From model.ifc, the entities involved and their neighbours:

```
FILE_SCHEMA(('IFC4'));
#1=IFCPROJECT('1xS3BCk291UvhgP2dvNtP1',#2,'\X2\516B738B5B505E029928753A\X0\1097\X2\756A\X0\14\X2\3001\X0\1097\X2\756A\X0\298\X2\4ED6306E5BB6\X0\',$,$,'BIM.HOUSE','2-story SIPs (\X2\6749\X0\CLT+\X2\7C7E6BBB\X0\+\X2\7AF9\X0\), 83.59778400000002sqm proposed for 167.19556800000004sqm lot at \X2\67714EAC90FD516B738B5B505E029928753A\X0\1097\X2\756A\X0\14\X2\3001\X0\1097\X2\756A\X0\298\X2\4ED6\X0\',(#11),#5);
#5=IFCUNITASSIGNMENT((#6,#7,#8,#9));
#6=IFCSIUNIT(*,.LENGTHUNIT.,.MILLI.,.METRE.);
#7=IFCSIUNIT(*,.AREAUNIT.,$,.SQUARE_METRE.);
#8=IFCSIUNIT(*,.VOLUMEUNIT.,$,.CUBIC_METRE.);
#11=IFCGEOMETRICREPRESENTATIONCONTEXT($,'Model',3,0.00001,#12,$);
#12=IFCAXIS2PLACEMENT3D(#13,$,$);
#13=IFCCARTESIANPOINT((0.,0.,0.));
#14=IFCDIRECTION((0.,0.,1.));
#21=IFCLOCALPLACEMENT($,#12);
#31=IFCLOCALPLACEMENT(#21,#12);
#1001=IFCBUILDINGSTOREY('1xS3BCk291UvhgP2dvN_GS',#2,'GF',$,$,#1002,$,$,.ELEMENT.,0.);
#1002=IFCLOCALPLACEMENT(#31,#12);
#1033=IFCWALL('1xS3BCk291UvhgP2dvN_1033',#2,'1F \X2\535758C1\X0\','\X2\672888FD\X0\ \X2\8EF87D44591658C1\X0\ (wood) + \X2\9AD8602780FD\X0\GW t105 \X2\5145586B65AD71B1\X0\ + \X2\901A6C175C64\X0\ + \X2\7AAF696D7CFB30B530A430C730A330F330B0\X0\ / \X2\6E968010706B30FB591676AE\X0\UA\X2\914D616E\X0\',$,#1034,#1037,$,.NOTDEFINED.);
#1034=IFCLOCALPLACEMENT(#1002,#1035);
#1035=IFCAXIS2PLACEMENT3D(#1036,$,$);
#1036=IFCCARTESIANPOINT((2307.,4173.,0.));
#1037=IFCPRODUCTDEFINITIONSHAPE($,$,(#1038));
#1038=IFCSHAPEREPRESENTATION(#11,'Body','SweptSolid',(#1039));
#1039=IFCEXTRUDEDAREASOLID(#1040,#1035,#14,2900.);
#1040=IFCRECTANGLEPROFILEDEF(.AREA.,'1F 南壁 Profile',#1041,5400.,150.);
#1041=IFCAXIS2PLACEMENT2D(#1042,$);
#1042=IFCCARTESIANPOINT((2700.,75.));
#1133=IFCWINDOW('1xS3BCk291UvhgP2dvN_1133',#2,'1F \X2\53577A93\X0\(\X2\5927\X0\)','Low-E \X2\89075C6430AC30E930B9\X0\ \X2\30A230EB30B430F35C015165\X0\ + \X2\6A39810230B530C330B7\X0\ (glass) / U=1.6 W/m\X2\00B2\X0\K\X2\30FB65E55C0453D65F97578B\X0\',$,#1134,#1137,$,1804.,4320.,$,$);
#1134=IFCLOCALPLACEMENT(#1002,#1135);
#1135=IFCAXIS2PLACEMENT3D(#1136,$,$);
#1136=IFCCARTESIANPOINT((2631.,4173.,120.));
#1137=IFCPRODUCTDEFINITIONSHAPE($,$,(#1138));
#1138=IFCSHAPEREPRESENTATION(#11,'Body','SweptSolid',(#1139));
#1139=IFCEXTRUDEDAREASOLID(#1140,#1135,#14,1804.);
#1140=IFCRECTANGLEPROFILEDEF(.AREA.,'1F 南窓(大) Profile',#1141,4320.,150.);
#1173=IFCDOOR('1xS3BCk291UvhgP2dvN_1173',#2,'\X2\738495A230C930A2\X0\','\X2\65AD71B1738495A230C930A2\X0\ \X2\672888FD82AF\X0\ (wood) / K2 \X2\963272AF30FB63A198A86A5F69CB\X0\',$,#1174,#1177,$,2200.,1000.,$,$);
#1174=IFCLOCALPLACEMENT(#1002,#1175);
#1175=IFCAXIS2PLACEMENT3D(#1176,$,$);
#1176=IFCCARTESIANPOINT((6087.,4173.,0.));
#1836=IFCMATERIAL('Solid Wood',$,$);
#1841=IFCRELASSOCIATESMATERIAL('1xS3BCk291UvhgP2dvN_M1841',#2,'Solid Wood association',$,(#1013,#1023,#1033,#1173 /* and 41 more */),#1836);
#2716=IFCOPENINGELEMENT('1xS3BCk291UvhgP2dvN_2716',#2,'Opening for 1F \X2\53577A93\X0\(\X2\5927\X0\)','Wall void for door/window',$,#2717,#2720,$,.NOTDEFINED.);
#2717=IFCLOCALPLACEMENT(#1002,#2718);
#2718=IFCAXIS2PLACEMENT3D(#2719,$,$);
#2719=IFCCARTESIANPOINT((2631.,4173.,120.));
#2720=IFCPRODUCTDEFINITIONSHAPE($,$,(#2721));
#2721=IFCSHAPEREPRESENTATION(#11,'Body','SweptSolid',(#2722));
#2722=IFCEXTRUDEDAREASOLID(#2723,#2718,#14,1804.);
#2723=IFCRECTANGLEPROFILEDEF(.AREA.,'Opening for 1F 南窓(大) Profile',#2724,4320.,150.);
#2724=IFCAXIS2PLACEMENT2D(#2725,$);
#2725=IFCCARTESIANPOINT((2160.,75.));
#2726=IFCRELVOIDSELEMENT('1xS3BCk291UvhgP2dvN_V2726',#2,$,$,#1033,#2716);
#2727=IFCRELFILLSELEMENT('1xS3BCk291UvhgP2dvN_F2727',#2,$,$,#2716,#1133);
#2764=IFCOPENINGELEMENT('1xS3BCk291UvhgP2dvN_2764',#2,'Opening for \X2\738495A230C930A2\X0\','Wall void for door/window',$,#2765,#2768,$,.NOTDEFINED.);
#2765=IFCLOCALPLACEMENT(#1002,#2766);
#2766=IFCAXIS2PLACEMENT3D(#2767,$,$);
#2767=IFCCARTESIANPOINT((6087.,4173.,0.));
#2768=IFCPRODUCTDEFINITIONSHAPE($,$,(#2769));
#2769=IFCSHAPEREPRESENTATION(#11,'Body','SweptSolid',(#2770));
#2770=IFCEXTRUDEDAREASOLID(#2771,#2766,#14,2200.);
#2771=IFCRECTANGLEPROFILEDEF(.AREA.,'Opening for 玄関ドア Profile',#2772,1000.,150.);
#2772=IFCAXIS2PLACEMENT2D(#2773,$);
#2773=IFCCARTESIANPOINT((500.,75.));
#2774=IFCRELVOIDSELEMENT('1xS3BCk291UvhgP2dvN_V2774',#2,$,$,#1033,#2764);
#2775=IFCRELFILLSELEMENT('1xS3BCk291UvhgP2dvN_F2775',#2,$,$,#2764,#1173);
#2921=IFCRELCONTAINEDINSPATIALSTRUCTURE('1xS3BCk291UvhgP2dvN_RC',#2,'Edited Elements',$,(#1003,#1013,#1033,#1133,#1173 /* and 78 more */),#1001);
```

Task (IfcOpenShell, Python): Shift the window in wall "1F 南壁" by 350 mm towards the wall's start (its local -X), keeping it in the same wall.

```python
import ifcopenshell
import ifcopenshell.api.geometry
import ifcopenshell.util.placement

model = ifcopenshell.open("model.ifc")

window = model.by_guid("1xS3BCk291UvhgP2dvN_1133")
opening = window.FillsVoids[0].RelatingOpeningElement
wall = opening.VoidsElements[0].RelatingBuildingElement

wall_matrix = ifcopenshell.util.placement.get_local_placement(wall.ObjectPlacement)
shift = wall_matrix[:3, 0] * -350.0
before = ifcopenshell.util.placement.get_local_placement(window.ObjectPlacement)[:3, 3].copy()

# The window is not placed relative to its opening, so move both.
for product in (opening, window):
    matrix = ifcopenshell.util.placement.get_local_placement(product.ObjectPlacement)
    matrix[:3, 3] += shift
    ifcopenshell.api.geometry.edit_object_placement(model, product=product, matrix=matrix, is_si=False)

after = ifcopenshell.util.placement.get_local_placement(window.ObjectPlacement)[:3, 3]
print("window moved by", (after - before).round(3) + 0.0)

model.write("model_updated.ifc")
```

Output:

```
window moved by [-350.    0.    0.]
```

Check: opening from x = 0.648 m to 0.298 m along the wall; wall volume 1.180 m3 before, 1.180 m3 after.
